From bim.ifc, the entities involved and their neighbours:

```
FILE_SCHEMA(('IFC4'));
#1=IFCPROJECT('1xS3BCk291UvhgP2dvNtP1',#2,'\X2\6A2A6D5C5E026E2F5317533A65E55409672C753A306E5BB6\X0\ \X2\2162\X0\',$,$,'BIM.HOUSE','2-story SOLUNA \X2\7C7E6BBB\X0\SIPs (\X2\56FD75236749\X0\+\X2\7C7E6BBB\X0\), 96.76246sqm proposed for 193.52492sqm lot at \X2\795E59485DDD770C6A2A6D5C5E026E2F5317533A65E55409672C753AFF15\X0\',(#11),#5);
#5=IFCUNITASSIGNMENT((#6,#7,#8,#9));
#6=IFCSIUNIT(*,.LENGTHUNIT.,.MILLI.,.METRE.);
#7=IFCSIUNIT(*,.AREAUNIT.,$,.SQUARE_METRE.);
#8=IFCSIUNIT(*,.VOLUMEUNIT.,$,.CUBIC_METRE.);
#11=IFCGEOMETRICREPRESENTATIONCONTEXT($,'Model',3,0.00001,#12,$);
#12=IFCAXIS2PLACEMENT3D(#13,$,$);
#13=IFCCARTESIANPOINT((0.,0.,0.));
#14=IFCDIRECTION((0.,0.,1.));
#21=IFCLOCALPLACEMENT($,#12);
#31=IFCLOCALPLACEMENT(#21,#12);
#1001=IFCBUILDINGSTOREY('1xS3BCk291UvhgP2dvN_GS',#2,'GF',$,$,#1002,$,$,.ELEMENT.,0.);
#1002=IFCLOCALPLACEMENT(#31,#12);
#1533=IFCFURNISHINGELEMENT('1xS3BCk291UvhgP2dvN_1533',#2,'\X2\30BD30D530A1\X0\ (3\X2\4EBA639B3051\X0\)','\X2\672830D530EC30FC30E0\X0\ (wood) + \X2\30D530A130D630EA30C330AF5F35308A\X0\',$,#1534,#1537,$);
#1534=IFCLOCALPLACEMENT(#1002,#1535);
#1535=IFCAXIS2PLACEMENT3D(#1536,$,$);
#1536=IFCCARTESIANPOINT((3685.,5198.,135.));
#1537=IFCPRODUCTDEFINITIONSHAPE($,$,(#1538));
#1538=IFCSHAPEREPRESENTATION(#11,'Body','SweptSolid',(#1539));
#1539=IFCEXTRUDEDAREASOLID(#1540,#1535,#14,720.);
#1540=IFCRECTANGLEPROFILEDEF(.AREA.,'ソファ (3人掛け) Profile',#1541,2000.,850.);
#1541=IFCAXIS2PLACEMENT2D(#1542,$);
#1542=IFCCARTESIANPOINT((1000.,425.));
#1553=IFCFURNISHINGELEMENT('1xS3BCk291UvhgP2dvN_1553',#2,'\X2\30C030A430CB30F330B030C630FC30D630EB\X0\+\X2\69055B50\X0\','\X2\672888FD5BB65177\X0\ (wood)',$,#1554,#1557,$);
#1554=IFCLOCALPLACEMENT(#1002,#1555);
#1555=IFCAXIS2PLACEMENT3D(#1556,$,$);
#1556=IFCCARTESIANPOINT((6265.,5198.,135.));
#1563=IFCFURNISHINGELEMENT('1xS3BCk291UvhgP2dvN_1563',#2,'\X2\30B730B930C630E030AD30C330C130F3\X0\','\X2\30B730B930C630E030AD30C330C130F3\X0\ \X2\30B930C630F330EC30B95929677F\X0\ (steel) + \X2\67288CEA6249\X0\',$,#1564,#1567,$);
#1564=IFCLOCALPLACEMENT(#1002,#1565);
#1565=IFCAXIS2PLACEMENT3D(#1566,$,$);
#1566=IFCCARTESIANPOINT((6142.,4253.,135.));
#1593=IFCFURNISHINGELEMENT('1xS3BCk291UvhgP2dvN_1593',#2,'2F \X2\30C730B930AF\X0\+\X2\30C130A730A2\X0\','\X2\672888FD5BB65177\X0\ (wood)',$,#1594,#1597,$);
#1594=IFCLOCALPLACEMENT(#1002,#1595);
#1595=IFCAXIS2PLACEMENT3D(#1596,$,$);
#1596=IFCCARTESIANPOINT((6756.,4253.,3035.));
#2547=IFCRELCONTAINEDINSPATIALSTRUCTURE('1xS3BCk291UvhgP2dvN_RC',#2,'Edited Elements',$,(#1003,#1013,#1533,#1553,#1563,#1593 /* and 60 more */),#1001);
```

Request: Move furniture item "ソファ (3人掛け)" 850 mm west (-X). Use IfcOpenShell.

```python
import ifcopenshell
import ifcopenshell.api.geometry
import ifcopenshell.util.placement

model = ifcopenshell.open("bim.ifc")

item = model.by_guid("1xS3BCk291UvhgP2dvN_1533")
matrix = ifcopenshell.util.placement.get_local_placement(item.ObjectPlacement)
matrix[0, 3] -= 850.0
ifcopenshell.api.geometry.edit_object_placement(model, product=item, matrix=matrix, is_si=False)

print(ifcopenshell.util.placement.get_local_placement(item.ObjectPlacement).round(3) + 0.0)

model.write("bim-out.ifc")
```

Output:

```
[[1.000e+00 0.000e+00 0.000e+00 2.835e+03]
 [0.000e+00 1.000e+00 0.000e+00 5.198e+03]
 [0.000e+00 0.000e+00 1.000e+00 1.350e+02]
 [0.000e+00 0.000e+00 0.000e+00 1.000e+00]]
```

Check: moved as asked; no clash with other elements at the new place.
